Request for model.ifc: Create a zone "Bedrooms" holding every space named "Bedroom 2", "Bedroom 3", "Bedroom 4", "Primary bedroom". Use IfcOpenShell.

First a look at what the model holds.

```python
import ifcopenshell

model = ifcopenshell.open("model.ifc")
print(model.schema)
seen = {}
for space in model.by_type("IfcSpace"):
    seen[space.LongName] = seen.get(space.LongName, 0) + 1
for name, count in sorted(seen.items(), key=str):
    print(count, "x", name)
print("zones:", [z.Name for z in model.by_type("IfcZone")][:20])
```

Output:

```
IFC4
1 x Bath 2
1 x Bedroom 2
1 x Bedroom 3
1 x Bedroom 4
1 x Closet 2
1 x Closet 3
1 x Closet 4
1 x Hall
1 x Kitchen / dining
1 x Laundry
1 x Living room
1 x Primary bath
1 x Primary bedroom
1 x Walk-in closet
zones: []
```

```python
import ifcopenshell
import ifcopenshell.api.group
import ifcopenshell.api.root

model = ifcopenshell.open("model.ifc")

names = {"Bedroom 2", "Bedroom 3", "Bedroom 4", "Primary bedroom"}
spaces = [s for s in model.by_type("IfcSpace") if s.LongName in names]

zone = ifcopenshell.api.root.create_entity(model, ifc_class="IfcZone", name="Bedrooms")
ifcopenshell.api.group.assign_group(model, products=spaces, group=zone)
print(len(spaces), "spaces in", zone.Name)

model.write("model_updated.ifc")
```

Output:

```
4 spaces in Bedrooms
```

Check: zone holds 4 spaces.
